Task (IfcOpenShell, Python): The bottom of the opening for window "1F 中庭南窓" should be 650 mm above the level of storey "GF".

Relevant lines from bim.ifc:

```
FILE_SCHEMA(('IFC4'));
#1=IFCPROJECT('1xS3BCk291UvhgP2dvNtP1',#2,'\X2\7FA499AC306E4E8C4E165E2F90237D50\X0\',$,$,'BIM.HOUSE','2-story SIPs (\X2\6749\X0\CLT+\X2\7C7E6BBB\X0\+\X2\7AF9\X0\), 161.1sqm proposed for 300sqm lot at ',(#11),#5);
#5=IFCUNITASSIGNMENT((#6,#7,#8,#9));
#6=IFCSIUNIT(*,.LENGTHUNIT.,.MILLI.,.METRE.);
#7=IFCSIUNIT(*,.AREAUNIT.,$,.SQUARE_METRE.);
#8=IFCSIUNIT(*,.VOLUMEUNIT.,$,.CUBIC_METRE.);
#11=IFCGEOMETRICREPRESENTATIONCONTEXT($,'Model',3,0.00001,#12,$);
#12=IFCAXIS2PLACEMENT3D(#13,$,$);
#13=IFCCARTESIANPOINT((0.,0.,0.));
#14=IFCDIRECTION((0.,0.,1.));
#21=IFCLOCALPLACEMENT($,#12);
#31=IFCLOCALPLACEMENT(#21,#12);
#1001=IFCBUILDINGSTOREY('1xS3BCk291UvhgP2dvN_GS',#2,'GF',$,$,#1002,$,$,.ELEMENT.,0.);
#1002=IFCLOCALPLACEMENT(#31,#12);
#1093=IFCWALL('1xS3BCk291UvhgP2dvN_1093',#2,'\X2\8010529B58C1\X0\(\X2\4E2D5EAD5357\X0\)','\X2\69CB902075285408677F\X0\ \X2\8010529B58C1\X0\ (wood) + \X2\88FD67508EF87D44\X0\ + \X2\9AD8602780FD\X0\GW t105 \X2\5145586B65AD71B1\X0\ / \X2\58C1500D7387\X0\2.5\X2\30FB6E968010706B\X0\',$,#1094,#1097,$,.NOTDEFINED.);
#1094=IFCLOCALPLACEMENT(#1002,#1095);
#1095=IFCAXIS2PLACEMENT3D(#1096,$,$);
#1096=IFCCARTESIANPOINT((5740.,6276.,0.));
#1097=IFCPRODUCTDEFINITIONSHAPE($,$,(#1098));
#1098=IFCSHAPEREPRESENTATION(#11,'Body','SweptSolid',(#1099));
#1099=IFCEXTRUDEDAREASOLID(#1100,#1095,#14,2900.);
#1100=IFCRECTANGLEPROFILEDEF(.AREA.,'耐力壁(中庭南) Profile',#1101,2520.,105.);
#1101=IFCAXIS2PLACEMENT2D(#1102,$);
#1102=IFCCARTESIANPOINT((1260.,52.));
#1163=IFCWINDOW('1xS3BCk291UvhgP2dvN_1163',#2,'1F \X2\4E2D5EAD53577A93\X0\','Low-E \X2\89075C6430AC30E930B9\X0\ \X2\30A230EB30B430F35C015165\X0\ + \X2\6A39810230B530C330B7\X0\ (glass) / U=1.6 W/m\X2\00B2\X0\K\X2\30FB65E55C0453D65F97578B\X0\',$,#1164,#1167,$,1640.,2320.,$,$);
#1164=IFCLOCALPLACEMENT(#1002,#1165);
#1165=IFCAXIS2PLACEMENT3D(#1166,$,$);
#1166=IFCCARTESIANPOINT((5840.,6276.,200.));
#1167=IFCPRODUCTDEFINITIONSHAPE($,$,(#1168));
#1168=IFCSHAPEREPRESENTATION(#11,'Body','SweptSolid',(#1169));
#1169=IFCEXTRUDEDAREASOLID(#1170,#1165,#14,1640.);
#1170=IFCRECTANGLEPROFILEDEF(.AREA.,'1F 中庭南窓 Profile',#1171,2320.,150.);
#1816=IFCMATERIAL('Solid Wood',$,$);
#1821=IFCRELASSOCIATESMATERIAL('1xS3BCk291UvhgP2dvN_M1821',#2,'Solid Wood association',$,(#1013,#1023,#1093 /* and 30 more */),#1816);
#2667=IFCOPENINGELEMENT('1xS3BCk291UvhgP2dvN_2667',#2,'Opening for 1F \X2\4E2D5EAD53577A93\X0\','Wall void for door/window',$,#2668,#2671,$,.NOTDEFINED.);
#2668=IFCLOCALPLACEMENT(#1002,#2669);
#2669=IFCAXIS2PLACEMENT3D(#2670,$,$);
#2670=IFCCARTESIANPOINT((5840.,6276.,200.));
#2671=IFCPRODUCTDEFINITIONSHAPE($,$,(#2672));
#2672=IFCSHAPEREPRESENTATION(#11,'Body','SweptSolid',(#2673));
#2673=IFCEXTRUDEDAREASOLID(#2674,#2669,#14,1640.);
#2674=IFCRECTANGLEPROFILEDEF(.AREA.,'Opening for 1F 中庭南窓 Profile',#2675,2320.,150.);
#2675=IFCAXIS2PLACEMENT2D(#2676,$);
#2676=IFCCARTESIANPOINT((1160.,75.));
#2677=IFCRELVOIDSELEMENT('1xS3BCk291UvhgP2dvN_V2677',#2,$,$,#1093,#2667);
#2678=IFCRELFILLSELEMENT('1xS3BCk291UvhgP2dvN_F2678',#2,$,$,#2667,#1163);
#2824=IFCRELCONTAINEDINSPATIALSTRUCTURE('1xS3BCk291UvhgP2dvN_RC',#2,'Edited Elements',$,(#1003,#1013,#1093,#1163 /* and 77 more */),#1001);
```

```python
import numpy as np
import ifcopenshell
import ifcopenshell.api.geometry
import ifcopenshell.geom
import ifcopenshell.util.element
import ifcopenshell.util.placement
import ifcopenshell.util.shape
import ifcopenshell.util.unit

model = ifcopenshell.open("bim.ifc")
unit_scale = ifcopenshell.util.unit.calculate_unit_scale(model)

window = model.by_guid("1xS3BCk291UvhgP2dvN_1163")
opening = window.FillsVoids[0].RelatingOpeningElement
storey = ifcopenshell.util.element.get_container(window, ifc_class="IfcBuildingStorey")
level = ifcopenshell.util.placement.get_local_placement(storey.ObjectPlacement)[2, 3]

# The opening's origin need not be at the sill, so measure its lowest point.
shape = ifcopenshell.geom.create_shape(ifcopenshell.geom.settings(), opening)
bottom = ifcopenshell.util.shape.get_shape_bottom_elevation(shape, shape.geometry) / unit_scale
dz = level + 650.0 - bottom

shift = np.array([0.0, 0.0, dz])
# The window is not placed relative to its opening, so move both.
for product in (opening, window):
    matrix = ifcopenshell.util.placement.get_local_placement(product.ObjectPlacement)
    matrix[:3, 3] += shift
    ifcopenshell.api.geometry.edit_object_placement(model, product=product, matrix=matrix, is_si=False)

print(f"moved by {dz * unit_scale:+.3f} m")

model.write("bim_rev.ifc")
```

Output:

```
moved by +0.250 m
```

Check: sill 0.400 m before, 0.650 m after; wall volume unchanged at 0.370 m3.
